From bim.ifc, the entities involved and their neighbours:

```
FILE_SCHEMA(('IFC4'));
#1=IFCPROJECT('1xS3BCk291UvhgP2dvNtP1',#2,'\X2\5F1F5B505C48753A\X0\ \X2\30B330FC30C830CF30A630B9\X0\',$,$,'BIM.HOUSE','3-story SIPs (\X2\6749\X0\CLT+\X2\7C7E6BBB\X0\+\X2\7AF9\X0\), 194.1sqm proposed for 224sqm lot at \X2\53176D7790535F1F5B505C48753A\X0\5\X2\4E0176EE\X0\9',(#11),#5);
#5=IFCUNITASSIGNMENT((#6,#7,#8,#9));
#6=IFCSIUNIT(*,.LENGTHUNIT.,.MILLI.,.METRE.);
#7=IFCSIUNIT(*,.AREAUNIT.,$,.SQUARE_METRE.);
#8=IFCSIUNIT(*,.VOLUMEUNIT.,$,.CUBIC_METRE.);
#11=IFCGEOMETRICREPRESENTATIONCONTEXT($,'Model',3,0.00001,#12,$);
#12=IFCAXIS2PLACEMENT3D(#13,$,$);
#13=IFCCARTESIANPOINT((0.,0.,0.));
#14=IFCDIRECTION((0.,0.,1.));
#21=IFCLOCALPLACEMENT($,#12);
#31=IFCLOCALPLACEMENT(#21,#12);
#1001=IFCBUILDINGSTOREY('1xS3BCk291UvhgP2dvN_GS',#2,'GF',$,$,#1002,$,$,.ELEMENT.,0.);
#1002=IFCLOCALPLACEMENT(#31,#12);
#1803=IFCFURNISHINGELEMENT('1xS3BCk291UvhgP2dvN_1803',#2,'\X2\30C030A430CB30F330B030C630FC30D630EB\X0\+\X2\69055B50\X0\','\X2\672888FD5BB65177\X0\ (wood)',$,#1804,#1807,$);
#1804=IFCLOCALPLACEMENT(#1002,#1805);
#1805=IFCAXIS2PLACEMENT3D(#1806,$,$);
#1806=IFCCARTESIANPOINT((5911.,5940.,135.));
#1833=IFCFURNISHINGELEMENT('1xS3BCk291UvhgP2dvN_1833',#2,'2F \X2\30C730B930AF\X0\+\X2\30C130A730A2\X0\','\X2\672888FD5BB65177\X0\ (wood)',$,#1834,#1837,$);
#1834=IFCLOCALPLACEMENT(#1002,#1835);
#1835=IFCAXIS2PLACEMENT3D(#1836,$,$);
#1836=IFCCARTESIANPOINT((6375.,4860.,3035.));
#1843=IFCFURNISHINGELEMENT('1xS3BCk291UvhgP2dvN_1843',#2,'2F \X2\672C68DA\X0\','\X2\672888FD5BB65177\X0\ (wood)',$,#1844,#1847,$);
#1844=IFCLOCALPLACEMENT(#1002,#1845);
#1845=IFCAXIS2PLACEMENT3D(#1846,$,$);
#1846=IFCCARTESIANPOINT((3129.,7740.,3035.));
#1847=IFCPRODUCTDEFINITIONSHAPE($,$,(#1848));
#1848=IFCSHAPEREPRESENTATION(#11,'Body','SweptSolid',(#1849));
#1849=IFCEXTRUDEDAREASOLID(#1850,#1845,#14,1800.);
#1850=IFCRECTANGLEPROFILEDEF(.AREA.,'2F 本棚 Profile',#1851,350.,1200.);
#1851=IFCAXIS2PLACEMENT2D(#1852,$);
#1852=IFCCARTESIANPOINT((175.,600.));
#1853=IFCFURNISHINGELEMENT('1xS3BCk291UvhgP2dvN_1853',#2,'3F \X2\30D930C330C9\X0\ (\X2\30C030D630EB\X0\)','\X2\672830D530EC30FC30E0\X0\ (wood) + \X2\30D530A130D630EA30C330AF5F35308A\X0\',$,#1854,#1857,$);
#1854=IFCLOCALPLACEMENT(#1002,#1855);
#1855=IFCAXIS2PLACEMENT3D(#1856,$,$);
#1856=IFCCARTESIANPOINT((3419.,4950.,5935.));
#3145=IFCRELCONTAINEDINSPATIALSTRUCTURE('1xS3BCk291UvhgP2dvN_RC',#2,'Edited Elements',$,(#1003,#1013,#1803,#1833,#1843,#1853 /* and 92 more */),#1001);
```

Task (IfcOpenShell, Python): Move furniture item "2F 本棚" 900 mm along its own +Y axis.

```python
import ifcopenshell
import ifcopenshell.api.geometry
import ifcopenshell.util.placement
import ifcopenshell.util.unit

model = ifcopenshell.open("bim.ifc")
unit_scale = ifcopenshell.util.unit.calculate_unit_scale(model)

item = model.by_guid("1xS3BCk291UvhgP2dvN_1843")
matrix = ifcopenshell.util.placement.get_local_placement(item.ObjectPlacement)
matrix[:3, 3] += matrix[:3, 1] * 0.9 / unit_scale
ifcopenshell.api.geometry.edit_object_placement(model, product=item, matrix=matrix, is_si=False)

print(ifcopenshell.util.placement.get_local_placement(item.ObjectPlacement).round(3) + 0.0)

model.write("bim_edited.ifc")
```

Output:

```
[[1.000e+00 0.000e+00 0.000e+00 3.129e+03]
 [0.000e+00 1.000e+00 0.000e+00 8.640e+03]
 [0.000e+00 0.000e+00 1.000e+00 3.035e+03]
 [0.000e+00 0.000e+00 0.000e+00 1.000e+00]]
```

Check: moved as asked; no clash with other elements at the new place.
